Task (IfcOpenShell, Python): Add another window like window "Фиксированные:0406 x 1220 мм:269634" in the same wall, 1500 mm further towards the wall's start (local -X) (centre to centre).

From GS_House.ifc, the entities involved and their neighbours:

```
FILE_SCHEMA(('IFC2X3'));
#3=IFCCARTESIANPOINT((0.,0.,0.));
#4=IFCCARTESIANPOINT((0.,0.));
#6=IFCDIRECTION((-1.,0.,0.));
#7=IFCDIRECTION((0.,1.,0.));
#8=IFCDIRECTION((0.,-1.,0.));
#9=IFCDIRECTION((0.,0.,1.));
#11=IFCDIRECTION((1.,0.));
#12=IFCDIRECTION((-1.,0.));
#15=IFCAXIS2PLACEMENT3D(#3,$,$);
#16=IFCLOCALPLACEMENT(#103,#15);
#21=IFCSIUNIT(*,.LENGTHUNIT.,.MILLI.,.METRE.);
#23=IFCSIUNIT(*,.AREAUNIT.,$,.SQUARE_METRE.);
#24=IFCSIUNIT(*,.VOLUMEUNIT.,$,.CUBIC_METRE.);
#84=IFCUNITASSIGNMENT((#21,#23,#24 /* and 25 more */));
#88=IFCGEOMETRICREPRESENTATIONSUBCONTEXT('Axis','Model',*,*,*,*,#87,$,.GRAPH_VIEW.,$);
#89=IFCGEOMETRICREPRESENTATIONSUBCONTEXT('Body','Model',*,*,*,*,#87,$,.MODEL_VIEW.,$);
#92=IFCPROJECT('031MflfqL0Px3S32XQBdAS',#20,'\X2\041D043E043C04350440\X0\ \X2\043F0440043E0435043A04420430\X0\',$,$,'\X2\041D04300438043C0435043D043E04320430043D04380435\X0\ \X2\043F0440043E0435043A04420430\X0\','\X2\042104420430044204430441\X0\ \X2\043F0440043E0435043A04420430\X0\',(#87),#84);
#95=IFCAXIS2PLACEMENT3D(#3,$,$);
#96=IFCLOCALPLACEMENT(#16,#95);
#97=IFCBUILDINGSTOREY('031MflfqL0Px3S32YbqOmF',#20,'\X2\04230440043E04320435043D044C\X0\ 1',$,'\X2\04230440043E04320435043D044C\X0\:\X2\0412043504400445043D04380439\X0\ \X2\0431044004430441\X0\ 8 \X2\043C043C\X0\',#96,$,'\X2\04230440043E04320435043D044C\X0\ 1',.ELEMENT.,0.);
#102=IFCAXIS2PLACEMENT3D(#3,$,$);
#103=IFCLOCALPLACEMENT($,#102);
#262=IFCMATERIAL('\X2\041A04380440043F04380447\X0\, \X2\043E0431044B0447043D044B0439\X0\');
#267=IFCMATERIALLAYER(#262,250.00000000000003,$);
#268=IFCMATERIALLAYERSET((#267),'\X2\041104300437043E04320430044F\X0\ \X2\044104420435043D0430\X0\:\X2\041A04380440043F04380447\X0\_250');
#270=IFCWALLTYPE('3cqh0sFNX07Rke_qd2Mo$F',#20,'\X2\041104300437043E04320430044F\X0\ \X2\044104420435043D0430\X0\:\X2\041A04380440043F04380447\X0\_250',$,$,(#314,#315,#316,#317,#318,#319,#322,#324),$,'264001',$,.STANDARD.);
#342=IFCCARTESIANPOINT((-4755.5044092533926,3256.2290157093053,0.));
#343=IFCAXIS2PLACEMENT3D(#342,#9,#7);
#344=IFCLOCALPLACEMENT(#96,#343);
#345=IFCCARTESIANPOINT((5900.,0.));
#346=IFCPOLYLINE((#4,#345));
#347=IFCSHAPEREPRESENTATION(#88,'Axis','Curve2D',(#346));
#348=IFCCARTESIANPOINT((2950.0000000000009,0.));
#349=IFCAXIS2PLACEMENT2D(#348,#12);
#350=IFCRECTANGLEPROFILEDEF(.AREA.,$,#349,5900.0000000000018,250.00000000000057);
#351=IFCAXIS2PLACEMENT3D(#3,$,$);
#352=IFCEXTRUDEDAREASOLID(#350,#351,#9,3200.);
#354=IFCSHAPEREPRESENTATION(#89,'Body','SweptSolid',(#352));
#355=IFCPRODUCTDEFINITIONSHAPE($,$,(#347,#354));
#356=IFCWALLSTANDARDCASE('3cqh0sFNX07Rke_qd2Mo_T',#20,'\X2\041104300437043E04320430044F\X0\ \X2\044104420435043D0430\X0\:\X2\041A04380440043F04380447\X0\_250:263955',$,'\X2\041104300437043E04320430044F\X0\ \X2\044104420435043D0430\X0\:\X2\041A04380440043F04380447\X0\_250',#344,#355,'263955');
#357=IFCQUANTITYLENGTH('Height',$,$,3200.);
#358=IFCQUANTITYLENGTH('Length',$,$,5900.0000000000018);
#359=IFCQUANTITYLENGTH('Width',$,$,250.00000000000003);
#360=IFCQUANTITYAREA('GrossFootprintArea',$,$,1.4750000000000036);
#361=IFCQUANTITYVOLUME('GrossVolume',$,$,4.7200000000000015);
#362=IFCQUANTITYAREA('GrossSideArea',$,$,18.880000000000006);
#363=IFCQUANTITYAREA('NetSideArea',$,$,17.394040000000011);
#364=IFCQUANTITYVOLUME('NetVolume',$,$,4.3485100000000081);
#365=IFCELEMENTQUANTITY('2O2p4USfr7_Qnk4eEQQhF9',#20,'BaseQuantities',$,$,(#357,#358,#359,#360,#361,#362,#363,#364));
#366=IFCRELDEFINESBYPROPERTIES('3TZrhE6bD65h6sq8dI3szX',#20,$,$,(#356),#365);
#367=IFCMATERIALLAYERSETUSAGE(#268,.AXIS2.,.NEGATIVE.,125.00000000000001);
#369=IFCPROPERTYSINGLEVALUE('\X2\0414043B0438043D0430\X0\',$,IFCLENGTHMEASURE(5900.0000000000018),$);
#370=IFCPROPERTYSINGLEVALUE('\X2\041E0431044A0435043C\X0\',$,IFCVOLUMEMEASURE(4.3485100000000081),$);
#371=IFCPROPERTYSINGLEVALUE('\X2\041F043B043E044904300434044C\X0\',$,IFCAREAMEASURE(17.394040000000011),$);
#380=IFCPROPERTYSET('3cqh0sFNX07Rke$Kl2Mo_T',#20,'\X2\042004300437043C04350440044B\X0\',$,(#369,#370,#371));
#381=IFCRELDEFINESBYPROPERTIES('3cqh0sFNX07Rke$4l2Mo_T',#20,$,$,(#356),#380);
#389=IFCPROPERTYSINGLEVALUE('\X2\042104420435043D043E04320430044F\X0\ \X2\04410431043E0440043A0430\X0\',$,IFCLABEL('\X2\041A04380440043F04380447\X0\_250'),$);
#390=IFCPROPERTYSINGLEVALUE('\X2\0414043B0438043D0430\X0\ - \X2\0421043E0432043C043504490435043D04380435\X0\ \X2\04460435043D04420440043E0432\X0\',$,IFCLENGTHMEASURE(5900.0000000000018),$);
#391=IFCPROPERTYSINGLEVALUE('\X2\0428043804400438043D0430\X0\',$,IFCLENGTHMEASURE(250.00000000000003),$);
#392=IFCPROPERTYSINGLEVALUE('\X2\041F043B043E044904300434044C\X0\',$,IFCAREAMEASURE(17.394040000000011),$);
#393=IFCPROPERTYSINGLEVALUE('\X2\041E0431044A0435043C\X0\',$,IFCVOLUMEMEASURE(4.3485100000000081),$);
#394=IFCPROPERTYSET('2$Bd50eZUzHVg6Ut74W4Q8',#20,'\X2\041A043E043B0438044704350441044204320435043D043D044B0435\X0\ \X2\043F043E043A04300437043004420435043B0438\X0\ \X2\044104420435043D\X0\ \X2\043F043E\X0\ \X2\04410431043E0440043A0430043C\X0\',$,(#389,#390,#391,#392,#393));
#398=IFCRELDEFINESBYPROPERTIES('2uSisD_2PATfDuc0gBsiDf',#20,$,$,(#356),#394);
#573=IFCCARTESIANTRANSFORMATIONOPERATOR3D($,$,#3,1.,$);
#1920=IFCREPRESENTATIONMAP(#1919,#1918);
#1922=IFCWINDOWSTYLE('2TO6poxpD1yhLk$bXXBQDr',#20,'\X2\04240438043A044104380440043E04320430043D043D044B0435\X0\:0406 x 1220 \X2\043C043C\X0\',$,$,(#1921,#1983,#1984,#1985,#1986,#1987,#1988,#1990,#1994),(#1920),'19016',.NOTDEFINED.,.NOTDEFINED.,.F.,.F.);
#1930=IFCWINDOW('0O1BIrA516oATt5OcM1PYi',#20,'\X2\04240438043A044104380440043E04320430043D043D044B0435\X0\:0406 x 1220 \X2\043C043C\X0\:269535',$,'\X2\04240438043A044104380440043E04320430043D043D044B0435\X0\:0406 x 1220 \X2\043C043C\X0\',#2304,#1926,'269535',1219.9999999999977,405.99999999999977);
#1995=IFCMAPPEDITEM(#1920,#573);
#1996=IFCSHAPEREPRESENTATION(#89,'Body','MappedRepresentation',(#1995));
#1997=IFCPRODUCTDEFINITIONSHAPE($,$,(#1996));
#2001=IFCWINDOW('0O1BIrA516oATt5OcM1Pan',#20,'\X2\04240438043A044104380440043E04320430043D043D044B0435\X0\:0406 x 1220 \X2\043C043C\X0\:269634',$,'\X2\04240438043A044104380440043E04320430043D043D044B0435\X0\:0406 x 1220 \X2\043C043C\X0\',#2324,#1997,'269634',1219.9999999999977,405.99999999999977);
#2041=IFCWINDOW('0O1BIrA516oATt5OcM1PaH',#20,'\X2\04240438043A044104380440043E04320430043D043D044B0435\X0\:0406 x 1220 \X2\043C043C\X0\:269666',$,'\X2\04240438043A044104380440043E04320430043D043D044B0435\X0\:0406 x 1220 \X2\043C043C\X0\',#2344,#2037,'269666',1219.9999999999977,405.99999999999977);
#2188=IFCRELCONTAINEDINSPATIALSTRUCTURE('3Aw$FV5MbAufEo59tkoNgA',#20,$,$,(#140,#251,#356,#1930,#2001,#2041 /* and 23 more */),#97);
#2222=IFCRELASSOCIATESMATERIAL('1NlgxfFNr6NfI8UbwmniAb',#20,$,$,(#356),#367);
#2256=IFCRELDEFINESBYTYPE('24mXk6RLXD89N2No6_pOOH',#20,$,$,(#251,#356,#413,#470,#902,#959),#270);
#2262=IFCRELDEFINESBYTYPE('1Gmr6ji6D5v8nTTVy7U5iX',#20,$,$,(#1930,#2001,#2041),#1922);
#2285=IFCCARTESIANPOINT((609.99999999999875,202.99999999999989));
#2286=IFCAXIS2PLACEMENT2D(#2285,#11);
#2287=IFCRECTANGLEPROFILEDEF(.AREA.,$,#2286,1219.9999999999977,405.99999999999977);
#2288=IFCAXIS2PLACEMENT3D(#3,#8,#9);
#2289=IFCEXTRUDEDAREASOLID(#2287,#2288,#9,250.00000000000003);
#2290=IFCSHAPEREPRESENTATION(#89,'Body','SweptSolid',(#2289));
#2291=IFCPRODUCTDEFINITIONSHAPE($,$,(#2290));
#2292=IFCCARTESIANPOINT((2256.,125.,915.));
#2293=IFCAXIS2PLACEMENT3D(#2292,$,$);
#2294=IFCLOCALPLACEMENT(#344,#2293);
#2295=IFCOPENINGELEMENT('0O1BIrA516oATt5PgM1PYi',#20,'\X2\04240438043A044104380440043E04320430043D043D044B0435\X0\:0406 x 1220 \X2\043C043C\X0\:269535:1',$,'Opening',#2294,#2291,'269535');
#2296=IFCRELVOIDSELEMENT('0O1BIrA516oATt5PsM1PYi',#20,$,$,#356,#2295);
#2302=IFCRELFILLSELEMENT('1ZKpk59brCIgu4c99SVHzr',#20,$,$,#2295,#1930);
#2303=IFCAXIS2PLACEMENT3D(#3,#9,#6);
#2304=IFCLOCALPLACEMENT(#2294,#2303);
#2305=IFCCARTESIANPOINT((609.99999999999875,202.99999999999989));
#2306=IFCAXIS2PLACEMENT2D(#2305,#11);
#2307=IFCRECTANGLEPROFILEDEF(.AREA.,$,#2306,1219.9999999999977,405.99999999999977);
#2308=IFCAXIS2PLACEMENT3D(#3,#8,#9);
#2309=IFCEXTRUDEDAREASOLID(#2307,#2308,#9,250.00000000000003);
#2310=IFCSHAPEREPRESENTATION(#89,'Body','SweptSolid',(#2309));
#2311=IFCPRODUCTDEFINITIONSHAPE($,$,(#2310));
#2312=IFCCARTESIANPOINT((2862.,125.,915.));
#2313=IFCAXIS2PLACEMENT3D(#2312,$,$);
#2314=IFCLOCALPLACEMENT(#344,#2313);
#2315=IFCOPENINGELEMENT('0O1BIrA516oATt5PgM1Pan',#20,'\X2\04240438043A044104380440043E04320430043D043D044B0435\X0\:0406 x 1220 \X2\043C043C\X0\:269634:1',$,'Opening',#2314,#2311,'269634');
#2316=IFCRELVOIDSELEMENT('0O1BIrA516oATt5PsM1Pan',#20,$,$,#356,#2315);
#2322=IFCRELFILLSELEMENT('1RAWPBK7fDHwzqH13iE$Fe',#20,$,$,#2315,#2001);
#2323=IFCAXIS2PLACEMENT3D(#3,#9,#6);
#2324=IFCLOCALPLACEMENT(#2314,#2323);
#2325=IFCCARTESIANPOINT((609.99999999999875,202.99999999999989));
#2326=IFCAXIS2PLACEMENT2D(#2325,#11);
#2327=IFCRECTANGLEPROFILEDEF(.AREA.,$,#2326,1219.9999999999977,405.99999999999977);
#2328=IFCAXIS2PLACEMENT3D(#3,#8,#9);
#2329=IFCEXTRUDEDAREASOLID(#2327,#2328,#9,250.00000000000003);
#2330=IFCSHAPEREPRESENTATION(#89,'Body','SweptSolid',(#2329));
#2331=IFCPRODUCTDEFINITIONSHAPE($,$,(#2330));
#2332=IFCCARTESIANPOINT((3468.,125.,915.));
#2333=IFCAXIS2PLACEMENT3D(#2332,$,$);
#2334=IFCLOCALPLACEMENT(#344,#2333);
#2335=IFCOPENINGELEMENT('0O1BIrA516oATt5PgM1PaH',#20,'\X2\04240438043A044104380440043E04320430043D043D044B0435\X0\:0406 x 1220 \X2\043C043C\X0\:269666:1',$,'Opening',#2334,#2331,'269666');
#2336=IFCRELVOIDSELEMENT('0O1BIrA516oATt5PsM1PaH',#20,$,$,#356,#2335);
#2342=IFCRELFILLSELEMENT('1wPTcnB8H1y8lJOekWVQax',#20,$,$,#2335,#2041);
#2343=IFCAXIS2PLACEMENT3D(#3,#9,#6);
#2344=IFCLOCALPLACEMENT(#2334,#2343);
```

```python
import ifcopenshell
import ifcopenshell.api.feature
import ifcopenshell.api.geometry
import ifcopenshell.api.pset
import ifcopenshell.api.root
import ifcopenshell.geom
import ifcopenshell.util.element
import ifcopenshell.util.placement
import ifcopenshell.util.shape
import ifcopenshell.util.unit

model = ifcopenshell.open("GS_House.ifc")
unit_scale = ifcopenshell.util.unit.calculate_unit_scale(model)
area_scale = ifcopenshell.util.unit.calculate_unit_scale(model, "AREAUNIT")
volume_scale = ifcopenshell.util.unit.calculate_unit_scale(model, "VOLUMEUNIT")
settings = ifcopenshell.geom.settings()


def volume(element):
    """Net volume in cubic metres, openings subtracted."""
    shape = ifcopenshell.geom.create_shape(settings, element)
    return ifcopenshell.util.shape.get_volume(shape.geometry)


def reuse_history(source, copy):
    """copy_class also copies each property set's owner history, people and application; keep the originals."""
    for rel in copy.IsDefinedBy:
        if rel.is_a("IfcRelDefinesByProperties") and (history := rel.RelatingPropertyDefinition.OwnerHistory):
            rel.RelatingPropertyDefinition.OwnerHistory = source.OwnerHistory
            ifcopenshell.util.element.remove_deep2(model, history)


window = model.by_id(2001)
opening = window.FillsVoids[0].RelatingOpeningElement
wall = opening.VoidsElements[0].RelatingBuildingElement
before = volume(wall)
shift = ifcopenshell.util.placement.get_local_placement(wall.ObjectPlacement)[:3, 0] * -1.5 / unit_scale

# copy_class copies the void relationship, type, container and properties, but no geometry.
new_opening = ifcopenshell.api.root.copy_class(model, product=opening)
new_opening.Representation = ifcopenshell.util.element.copy_deep(
    model, opening.Representation, exclude=["IfcGeometricRepresentationContext", "IfcRepresentationMap"]
)
new_opening.Name = "Фиксированные:0406 x 1220 мм"
new_opening.Tag = None
reuse_history(opening, new_opening)
new_window = ifcopenshell.api.root.copy_class(model, product=window)
new_window.Representation = ifcopenshell.util.element.copy_deep(
    model, window.Representation, exclude=["IfcGeometricRepresentationContext", "IfcRepresentationMap"]
)
new_window.Name = "Фиксированные:0406 x 1220 мм"
new_window.Tag = None
reuse_history(window, new_window)
fills = ifcopenshell.api.feature.add_filling(model, opening=new_opening, element=new_window)
fills.OwnerHistory = new_window.OwnerHistory  # required in IFC2X3

for old, new in ((opening, new_opening), (window, new_window)):
    matrix = ifcopenshell.util.placement.get_local_placement(old.ObjectPlacement)
    matrix[:3, 3] += shift
    ifcopenshell.api.geometry.edit_object_placement(model, product=new, matrix=matrix, is_si=False)

after = volume(wall)
thickness = 0.25  # wall thickness in metres

# Update the wall's stored quantities.
qto = model.by_id(ifcopenshell.util.element.get_pset(wall, "BaseQuantities", should_inherit=False)["id"])
ifcopenshell.api.pset.edit_qto(model, qto=qto, properties={
    "NetSideArea": after / thickness / area_scale,
    "NetVolume": after / volume_scale,
})
pset = model.by_id(ifcopenshell.util.element.get_pset(wall, "Размеры", should_inherit=False)["id"])
ifcopenshell.api.pset.edit_pset(model, pset=pset, properties={
    "Объем": model.create_entity("IfcVolumeMeasure", after / volume_scale),
    "Площадь": model.create_entity("IfcAreaMeasure", after / thickness / area_scale),
})
pset = model.by_id(ifcopenshell.util.element.get_pset(wall, "Количественные показатели стен по сборкам", should_inherit=False)["id"])
ifcopenshell.api.pset.edit_pset(model, pset=pset, properties={
    "Площадь": model.create_entity("IfcAreaMeasure", after / thickness / area_scale),
    "Объем": model.create_entity("IfcVolumeMeasure", after / volume_scale),
})

print(f"wall volume {before:.3f} -> {after:.3f} m3")

model.write("GS_House_updated.ifc")
```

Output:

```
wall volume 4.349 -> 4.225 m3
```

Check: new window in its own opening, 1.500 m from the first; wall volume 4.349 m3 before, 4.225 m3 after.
